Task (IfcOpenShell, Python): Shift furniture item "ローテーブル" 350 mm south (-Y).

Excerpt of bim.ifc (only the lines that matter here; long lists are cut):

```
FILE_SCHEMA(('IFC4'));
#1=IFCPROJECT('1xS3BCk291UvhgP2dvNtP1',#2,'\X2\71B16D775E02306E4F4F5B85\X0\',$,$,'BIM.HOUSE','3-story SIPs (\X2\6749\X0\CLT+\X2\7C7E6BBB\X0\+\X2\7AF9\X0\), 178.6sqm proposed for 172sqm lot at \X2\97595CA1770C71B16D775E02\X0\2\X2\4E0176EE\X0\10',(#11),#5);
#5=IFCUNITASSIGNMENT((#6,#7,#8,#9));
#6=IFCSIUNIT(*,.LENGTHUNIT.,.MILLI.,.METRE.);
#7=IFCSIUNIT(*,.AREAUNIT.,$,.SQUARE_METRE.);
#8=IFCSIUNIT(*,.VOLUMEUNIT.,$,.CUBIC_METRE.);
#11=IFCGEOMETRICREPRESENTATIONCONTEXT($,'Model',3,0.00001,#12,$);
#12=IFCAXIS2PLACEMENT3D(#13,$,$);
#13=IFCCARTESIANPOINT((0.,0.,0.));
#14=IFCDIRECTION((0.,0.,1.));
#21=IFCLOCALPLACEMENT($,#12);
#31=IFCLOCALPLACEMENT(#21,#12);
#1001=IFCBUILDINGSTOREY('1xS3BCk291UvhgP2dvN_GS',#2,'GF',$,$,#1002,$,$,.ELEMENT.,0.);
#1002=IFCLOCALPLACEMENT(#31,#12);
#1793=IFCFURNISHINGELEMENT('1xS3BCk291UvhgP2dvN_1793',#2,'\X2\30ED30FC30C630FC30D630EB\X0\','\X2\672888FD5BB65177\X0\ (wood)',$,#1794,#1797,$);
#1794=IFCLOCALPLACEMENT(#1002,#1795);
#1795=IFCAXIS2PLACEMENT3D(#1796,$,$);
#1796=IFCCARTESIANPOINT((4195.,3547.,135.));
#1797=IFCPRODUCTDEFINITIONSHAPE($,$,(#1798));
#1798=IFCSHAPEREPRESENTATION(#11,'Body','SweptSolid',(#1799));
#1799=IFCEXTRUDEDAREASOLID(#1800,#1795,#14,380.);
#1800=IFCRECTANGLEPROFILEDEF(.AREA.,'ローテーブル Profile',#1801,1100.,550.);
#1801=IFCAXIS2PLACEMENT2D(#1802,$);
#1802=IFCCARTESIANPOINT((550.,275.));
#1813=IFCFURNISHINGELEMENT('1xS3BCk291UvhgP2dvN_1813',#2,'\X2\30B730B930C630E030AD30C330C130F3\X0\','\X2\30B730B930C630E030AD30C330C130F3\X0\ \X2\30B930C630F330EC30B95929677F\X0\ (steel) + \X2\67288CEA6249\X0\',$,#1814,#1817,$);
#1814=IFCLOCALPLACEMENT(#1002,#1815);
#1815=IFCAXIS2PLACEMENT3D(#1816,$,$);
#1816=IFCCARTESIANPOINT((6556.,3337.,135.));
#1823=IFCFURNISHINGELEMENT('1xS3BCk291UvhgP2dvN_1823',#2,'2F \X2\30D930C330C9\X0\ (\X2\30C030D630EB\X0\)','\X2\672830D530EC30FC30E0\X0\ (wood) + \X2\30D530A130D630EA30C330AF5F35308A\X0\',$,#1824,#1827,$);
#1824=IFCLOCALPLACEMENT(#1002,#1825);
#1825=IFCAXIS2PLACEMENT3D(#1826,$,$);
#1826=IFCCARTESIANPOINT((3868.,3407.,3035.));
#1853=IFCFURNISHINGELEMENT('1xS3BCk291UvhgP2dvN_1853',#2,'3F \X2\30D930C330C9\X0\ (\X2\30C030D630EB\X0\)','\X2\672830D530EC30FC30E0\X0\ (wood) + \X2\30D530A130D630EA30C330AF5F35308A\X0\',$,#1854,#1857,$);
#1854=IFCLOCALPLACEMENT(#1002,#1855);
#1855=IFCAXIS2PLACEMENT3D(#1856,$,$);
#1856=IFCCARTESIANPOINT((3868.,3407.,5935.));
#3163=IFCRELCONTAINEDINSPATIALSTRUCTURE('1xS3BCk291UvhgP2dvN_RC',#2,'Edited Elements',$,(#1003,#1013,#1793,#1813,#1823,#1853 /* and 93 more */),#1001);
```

```python
import ifcopenshell
import ifcopenshell.api.geometry
import ifcopenshell.util.placement
import ifcopenshell.util.unit

model = ifcopenshell.open("bim.ifc")
unit_scale = ifcopenshell.util.unit.calculate_unit_scale(model)

item = model.by_guid("1xS3BCk291UvhgP2dvN_1793")
matrix = ifcopenshell.util.placement.get_local_placement(item.ObjectPlacement)
matrix[1, 3] -= 0.35 / unit_scale
ifcopenshell.api.geometry.edit_object_placement(model, product=item, matrix=matrix, is_si=False)

print(ifcopenshell.util.placement.get_local_placement(item.ObjectPlacement).round(3) + 0.0)

model.write("bim_updated.ifc")
```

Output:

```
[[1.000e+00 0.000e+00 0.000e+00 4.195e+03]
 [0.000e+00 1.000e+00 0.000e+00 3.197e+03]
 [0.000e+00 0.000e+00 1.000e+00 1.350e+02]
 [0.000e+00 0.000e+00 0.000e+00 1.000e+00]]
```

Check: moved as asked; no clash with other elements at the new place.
